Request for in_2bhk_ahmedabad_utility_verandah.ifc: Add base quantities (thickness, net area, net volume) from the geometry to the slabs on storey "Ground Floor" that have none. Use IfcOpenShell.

First a look at what the model holds.

```python
import ifcopenshell
import ifcopenshell.util.element
import ifcopenshell.util.unit

model = ifcopenshell.open("in_2bhk_ahmedabad_utility_verandah.ifc")
print(model.schema)
for unit_type in ("LENGTHUNIT", "AREAUNIT", "VOLUMEUNIT"):
    print(unit_type, ifcopenshell.util.unit.calculate_unit_scale(model, unit_type))
storey = next(s for s in model.by_type("IfcBuildingStorey") if s.Name == "Ground Floor")
slabs = [e for e in ifcopenshell.util.element.get_decomposition(storey) if e.is_a("IfcSlab")]
for e in sorted(slabs, key=lambda e: e.id()):
    print(e.id(), e.is_a(), e.Name, list(ifcopenshell.util.element.get_psets(e, qtos_only=True)), sep=" | ")
```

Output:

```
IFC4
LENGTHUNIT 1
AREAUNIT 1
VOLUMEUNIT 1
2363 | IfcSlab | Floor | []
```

```python
import ifcopenshell
import ifcopenshell.api.pset
import ifcopenshell.geom
import ifcopenshell.util.element
import ifcopenshell.util.shape
import ifcopenshell.util.unit

model = ifcopenshell.open("in_2bhk_ahmedabad_utility_verandah.ifc")
unit_scale = ifcopenshell.util.unit.calculate_unit_scale(model)
area_scale = ifcopenshell.util.unit.calculate_unit_scale(model, "AREAUNIT")
volume_scale = ifcopenshell.util.unit.calculate_unit_scale(model, "VOLUMEUNIT")
settings = ifcopenshell.geom.settings()

storey = next(s for s in model.by_type("IfcBuildingStorey") if s.Name == "Ground Floor")
slabs = [e for e in ifcopenshell.util.element.get_decomposition(storey) if e.is_a("IfcSlab")]

for e in sorted(slabs, key=lambda e: e.id()):
    if ifcopenshell.util.element.get_psets(e, qtos_only=True, should_inherit=False):
        continue
    # Geometry comes back in metres, in the element's own axes.
    shape = ifcopenshell.geom.create_shape(settings, e)
    values = {
        "Width": ifcopenshell.util.shape.get_z(shape.geometry) / unit_scale,
        "NetArea": ifcopenshell.util.shape.get_footprint_area(shape.geometry) / area_scale,
        "NetVolume": ifcopenshell.util.shape.get_volume(shape.geometry) / volume_scale,
    }
    qto = ifcopenshell.api.pset.add_qto(model, product=e, name="Qto_SlabBaseQuantities")
    ifcopenshell.api.pset.edit_qto(model, qto=qto, properties=values)
    print(e.id(), {k: round(v, 3) for k, v in values.items()})

model.write("in_2bhk_ahmedabad_utility_verandah_v2.ifc")
```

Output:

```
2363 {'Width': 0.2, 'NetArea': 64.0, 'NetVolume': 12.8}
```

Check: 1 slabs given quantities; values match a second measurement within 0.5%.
